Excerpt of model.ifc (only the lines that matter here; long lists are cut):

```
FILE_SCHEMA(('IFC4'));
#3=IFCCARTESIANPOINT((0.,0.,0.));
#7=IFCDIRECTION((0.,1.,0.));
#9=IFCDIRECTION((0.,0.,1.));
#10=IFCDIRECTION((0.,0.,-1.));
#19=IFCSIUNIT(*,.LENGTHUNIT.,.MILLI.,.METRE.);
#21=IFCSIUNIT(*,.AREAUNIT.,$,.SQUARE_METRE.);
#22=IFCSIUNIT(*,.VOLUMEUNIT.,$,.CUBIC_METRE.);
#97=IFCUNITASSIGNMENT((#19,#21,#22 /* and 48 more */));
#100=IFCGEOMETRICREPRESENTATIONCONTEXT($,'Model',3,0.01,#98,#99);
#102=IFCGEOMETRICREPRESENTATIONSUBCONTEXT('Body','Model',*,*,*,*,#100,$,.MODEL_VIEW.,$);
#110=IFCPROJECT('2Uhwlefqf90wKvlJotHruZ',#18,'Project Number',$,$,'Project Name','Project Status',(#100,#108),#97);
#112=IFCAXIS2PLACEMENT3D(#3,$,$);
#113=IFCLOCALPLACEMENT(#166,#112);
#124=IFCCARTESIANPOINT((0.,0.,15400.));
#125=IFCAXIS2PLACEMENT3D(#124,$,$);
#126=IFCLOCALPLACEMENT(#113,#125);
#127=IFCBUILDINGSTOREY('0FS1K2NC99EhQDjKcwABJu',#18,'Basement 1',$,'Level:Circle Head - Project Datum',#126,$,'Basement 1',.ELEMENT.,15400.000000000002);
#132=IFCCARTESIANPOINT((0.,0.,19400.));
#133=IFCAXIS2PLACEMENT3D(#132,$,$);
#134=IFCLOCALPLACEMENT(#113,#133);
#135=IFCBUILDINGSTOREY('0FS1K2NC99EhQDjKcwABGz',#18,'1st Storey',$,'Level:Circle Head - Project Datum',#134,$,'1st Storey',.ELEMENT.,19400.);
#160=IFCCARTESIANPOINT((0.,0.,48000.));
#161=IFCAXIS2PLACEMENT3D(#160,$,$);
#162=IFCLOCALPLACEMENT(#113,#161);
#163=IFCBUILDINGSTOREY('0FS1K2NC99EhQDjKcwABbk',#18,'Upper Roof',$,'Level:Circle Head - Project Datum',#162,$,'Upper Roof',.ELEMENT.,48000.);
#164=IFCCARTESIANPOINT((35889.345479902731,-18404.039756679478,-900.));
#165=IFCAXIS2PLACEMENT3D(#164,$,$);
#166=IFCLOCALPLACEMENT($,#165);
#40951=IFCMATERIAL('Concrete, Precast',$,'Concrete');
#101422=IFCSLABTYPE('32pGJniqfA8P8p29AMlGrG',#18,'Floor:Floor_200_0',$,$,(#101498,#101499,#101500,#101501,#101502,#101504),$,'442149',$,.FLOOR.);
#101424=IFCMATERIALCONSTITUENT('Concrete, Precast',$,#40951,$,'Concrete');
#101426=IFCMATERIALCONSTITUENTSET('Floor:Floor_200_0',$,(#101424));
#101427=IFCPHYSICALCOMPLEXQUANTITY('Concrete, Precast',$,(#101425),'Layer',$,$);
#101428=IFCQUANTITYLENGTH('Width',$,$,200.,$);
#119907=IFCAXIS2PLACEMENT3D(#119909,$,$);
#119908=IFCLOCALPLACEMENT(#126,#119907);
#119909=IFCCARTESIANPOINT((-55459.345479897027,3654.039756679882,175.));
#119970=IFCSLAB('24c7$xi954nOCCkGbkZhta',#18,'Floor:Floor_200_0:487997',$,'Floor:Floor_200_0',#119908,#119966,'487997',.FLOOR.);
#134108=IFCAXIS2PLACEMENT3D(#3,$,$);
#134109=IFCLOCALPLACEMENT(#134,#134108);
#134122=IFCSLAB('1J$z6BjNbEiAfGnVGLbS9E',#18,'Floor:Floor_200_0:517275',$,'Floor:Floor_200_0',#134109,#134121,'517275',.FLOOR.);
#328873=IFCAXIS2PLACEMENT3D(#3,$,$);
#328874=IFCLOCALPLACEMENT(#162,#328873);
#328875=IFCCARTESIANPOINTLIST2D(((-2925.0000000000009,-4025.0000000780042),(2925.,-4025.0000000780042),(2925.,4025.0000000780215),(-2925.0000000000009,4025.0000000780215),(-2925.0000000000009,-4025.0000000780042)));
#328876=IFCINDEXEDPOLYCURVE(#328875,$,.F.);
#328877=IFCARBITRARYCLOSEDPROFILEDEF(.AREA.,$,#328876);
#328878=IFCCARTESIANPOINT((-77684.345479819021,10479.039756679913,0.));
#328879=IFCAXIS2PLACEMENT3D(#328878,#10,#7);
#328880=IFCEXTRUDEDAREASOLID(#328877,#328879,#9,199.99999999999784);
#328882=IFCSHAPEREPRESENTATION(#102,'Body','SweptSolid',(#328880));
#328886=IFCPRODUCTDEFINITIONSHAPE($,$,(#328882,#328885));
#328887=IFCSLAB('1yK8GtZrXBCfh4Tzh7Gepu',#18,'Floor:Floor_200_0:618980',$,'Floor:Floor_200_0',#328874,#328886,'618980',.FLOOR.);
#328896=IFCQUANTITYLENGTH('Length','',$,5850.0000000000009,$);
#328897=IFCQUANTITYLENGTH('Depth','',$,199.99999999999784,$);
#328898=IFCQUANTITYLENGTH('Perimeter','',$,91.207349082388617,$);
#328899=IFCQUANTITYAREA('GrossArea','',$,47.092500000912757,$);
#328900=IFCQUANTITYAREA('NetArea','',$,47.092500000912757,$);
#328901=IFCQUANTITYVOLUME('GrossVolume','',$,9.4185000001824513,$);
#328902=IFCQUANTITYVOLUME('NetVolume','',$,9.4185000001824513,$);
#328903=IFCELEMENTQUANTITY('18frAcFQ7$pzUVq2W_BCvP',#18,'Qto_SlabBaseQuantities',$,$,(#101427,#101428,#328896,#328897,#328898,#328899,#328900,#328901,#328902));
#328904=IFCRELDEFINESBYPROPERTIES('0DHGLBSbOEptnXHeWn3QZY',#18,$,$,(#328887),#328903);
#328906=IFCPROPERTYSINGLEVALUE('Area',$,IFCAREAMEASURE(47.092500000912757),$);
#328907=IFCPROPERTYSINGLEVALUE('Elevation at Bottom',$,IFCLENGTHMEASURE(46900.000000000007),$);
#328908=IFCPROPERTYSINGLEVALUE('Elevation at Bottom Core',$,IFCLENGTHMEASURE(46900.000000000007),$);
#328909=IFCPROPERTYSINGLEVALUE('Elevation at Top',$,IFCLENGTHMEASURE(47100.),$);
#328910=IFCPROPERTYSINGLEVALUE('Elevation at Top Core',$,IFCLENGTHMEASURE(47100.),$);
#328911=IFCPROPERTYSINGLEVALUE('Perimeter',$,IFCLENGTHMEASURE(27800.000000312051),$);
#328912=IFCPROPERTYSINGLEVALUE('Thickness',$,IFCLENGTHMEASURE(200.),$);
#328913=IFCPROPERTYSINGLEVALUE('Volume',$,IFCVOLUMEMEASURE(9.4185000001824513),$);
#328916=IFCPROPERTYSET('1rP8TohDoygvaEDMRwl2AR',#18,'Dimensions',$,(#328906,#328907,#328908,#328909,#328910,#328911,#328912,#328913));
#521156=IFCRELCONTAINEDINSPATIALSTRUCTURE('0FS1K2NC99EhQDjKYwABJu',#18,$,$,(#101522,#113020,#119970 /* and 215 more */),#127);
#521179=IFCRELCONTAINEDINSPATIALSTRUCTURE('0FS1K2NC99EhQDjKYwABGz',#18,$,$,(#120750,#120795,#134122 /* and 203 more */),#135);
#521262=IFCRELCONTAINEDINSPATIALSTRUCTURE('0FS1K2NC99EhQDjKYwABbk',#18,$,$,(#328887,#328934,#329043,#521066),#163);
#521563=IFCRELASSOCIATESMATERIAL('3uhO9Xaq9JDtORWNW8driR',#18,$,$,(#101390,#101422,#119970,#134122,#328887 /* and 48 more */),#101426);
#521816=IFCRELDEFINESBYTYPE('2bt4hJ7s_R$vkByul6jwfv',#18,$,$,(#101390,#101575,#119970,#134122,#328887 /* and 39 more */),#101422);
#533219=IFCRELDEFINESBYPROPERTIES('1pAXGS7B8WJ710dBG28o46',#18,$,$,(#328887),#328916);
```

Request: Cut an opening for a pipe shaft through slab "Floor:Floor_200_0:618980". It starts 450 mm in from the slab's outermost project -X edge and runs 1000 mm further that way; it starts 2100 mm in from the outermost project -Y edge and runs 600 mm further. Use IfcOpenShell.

```python
import numpy as np
import ifcopenshell
import ifcopenshell.api.feature
import ifcopenshell.api.geometry
import ifcopenshell.api.pset
import ifcopenshell.api.root
import ifcopenshell.geom
import ifcopenshell.util.element
import ifcopenshell.util.placement
import ifcopenshell.util.representation
import ifcopenshell.util.shape
import ifcopenshell.util.unit

model = ifcopenshell.open("model.ifc")
unit_scale = ifcopenshell.util.unit.calculate_unit_scale(model)
area_scale = ifcopenshell.util.unit.calculate_unit_scale(model, "AREAUNIT")
volume_scale = ifcopenshell.util.unit.calculate_unit_scale(model, "VOLUMEUNIT")
settings = ifcopenshell.geom.settings()


def volume(element):
    """Net volume in cubic metres, openings subtracted."""
    shape = ifcopenshell.geom.create_shape(settings, element)
    return ifcopenshell.util.shape.get_volume(shape.geometry)


slab = model.by_guid("1yK8GtZrXBCfh4Tzh7Gepu")
before = volume(slab)

# Extent in the slab's own axes, in metres. The edges named are its -X and -Y sides.
slab_shape = ifcopenshell.geom.create_shape(settings, slab)
vertices = ifcopenshell.util.shape.get_vertices(slab_shape.geometry)
x_min, y_min, bottom = vertices.min(axis=0)
top = vertices[:, 2].max()

opening = ifcopenshell.api.root.create_entity(model, ifc_class="IfcOpeningElement", name="Pipe shaft opening", predefined_type="OPENING")
context = ifcopenshell.util.representation.get_context(model, "Model", "Body", "MODEL_VIEW")
width, depth = 1, 0.6
outline = [(0.0, 0.0), (width, 0.0), (width, depth), (0.0, depth), (0.0, 0.0)]
# Overshoot both faces by 50 mm so the cut is clean.
shape = ifcopenshell.api.geometry.add_slab_representation(
    model, context=context, depth=top - bottom + 0.1, polyline=outline
)
ifcopenshell.api.geometry.assign_representation(model, product=opening, representation=shape)

matrix = ifcopenshell.util.placement.get_local_placement(slab.ObjectPlacement)
matrix[:, 3] = matrix @ np.append(np.array([x_min + 0.45, y_min + 2.1, bottom - 0.05]) / unit_scale, 1.0)
ifcopenshell.api.geometry.edit_object_placement(model, product=opening, matrix=matrix, is_si=False)
ifcopenshell.api.feature.add_feature(model, feature=opening, element=slab)

after = volume(slab)

# Update the slab's stored quantities.
qto = model.by_id(ifcopenshell.util.element.get_pset(slab, "Qto_SlabBaseQuantities", should_inherit=False)["id"])
ifcopenshell.api.pset.edit_qto(model, qto=qto, properties={
    "NetArea": after / (top - bottom) / area_scale,
    "NetVolume": after / volume_scale,
})
pset = model.by_id(ifcopenshell.util.element.get_pset(slab, "Dimensions", should_inherit=False)["id"])
ifcopenshell.api.pset.edit_pset(model, pset=pset, properties={
    "Area": model.create_entity("IfcAreaMeasure", after / (top - bottom) / area_scale),
    "Volume": model.create_entity("IfcVolumeMeasure", after / volume_scale),
})

print(f"slab volume {before:.3f} -> {after:.3f} m3")

model.write("model-out.ifc")
```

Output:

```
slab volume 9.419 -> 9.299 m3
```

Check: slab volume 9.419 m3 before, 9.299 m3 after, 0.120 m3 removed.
